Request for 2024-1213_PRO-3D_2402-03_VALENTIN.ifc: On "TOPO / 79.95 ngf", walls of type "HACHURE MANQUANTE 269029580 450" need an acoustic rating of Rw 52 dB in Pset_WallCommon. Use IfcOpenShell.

First a look at what the model holds.

```python
import ifcopenshell
import ifcopenshell.util.element

model = ifcopenshell.open("2024-1213_PRO-3D_2402-03_VALENTIN.ifc")
print(model.schema)
storey = next(s for s in model.by_type("IfcBuildingStorey") if s.Name == "TOPO / 79.95 ngf")
walls = [e for e in ifcopenshell.util.element.get_decomposition(storey) if e.is_a("IfcWall")]
seen = {}
for e in walls:
    element_type = ifcopenshell.util.element.get_type(e)
    key = (element_type.Name if element_type != e and element_type else None, ifcopenshell.util.element.get_pset(e, "Pset_WallCommon", "AcousticRating"))
    seen[key] = seen.get(key, 0) + 1
for (name, value), count in sorted(seen.items(), key=str):
    print(count, "x", name, "|", value)
```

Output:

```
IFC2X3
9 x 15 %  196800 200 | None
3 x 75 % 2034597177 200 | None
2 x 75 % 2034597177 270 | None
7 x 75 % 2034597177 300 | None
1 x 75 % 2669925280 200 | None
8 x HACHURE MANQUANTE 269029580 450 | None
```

```python
import ifcopenshell
import ifcopenshell.api.pset
import ifcopenshell.util.element

model = ifcopenshell.open("2024-1213_PRO-3D_2402-03_VALENTIN.ifc")

storey = next(s for s in model.by_type("IfcBuildingStorey") if s.Name == "TOPO / 79.95 ngf")
walls = [e for e in ifcopenshell.util.element.get_decomposition(storey) if e.is_a("IfcWall")]

count = 0
for e in walls:
    element_type = ifcopenshell.util.element.get_type(e)
    if element_type in (None, e) or element_type.Name != "HACHURE MANQUANTE 269029580 450":
        continue
    # add_pset returns the element's existing set when there is one.
    pset = ifcopenshell.api.pset.add_pset(model, product=e, name="Pset_WallCommon")
    ifcopenshell.api.pset.edit_pset(model, pset=pset, properties={"AcousticRating": "Rw 52 dB"})
    count += 1

print(count, "walls updated")

model.write("2024-1213_PRO-3D_2402-03_VALENTIN-out.ifc")
```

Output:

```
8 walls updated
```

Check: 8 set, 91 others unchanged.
